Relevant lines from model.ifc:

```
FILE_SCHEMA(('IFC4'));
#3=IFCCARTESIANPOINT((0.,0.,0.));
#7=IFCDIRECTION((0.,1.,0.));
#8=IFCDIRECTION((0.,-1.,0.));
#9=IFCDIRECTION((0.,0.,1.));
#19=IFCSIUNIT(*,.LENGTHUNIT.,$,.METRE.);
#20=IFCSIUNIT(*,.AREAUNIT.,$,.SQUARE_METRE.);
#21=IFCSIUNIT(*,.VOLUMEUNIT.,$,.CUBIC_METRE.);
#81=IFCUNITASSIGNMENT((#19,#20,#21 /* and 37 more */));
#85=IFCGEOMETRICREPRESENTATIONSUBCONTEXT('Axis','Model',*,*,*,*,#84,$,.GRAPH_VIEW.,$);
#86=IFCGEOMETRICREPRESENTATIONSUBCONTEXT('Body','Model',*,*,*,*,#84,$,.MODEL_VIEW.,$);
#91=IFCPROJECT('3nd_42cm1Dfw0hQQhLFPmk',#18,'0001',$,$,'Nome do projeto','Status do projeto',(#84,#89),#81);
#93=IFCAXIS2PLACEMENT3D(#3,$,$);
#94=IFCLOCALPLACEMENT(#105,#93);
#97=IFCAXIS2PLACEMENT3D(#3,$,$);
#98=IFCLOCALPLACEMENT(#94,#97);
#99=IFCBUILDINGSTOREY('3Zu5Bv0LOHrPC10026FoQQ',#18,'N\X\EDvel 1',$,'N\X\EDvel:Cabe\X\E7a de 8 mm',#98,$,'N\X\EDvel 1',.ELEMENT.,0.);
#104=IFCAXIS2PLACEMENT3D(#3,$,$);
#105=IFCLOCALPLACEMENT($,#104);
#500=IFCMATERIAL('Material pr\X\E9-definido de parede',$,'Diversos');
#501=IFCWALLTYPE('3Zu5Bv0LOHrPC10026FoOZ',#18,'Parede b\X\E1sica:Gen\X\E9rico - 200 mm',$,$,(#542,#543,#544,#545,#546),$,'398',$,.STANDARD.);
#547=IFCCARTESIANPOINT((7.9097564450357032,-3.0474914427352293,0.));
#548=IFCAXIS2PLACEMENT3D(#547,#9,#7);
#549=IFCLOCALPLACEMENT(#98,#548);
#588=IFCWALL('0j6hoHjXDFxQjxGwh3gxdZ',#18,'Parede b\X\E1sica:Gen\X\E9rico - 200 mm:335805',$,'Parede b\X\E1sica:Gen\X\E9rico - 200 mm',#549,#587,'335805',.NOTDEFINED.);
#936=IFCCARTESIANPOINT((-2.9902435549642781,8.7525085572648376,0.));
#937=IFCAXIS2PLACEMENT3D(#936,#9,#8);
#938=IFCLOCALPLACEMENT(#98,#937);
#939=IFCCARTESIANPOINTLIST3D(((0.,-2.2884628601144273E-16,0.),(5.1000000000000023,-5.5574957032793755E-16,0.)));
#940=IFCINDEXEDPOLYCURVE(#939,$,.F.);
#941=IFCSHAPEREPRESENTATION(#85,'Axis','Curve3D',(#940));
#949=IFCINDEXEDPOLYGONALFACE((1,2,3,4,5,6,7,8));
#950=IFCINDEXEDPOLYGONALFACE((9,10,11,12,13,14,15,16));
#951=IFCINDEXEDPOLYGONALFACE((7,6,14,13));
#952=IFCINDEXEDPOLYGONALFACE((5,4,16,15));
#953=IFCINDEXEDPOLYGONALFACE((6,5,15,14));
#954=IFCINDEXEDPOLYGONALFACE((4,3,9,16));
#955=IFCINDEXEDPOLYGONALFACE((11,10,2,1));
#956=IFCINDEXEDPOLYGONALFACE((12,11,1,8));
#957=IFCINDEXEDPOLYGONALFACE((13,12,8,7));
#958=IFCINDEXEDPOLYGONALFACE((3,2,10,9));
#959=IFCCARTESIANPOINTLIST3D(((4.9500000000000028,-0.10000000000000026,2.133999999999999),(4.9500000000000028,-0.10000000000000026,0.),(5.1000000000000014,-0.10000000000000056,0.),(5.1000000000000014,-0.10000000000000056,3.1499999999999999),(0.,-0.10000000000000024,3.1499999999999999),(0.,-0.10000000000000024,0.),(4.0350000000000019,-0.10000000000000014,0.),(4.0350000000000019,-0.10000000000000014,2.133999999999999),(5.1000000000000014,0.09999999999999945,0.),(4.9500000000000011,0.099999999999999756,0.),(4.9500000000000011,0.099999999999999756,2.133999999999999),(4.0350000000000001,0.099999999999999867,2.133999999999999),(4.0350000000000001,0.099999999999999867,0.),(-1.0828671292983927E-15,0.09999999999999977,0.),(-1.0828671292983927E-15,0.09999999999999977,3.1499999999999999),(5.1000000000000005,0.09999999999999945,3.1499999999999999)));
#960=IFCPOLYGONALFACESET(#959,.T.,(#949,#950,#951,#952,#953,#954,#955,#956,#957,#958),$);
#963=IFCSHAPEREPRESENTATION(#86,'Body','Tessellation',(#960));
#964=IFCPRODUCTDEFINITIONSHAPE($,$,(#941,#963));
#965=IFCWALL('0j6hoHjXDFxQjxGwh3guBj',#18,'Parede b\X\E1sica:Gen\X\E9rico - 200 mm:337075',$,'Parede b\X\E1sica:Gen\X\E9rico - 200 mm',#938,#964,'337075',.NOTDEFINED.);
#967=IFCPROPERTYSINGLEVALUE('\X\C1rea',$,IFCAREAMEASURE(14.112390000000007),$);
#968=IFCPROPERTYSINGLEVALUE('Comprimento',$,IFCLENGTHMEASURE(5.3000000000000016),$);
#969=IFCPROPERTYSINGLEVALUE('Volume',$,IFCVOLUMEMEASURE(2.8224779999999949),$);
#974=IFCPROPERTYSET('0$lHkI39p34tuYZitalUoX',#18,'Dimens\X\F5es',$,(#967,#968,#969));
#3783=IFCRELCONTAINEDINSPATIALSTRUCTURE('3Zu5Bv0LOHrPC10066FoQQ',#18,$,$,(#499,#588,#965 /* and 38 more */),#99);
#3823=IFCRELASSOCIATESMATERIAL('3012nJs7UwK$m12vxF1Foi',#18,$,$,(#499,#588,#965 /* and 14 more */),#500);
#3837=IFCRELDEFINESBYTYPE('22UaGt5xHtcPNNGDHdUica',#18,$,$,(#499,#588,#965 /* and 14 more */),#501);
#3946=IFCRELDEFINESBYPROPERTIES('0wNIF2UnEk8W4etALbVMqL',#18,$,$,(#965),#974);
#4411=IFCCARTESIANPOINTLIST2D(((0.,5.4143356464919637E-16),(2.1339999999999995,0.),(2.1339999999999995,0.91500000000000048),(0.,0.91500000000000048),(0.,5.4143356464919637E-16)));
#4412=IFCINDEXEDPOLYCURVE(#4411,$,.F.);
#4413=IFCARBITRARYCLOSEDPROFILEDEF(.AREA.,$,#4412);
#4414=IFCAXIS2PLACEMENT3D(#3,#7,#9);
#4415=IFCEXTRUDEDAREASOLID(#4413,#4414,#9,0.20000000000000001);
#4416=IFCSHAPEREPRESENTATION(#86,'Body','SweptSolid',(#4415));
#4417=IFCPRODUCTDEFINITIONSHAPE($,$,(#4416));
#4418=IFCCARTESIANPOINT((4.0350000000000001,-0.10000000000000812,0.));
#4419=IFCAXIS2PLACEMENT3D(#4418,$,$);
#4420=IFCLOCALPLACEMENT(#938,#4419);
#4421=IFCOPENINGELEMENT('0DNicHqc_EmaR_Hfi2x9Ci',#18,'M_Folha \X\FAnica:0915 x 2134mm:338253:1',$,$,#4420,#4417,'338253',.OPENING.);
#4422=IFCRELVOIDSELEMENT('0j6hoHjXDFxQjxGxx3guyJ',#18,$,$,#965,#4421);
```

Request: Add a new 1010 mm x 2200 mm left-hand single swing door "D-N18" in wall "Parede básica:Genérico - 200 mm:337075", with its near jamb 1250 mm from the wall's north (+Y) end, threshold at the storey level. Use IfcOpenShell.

```python
import numpy as np
import ifcopenshell
import ifcopenshell.api.feature
import ifcopenshell.api.geometry
import ifcopenshell.api.pset
import ifcopenshell.api.root
import ifcopenshell.api.spatial
import ifcopenshell.geom
import ifcopenshell.util.element
import ifcopenshell.util.placement
import ifcopenshell.util.representation
import ifcopenshell.util.shape
import ifcopenshell.util.unit

model = ifcopenshell.open("model.ifc")
unit_scale = ifcopenshell.util.unit.calculate_unit_scale(model)
area_scale = ifcopenshell.util.unit.calculate_unit_scale(model, "AREAUNIT")
volume_scale = ifcopenshell.util.unit.calculate_unit_scale(model, "VOLUMEUNIT")
settings = ifcopenshell.geom.settings()


def volume(element):
    """Net volume in cubic metres, openings subtracted."""
    shape = ifcopenshell.geom.create_shape(settings, element)
    return ifcopenshell.util.shape.get_volume(shape.geometry)


wall = model.by_guid("0j6hoHjXDFxQjxGwh3guBj")
storey = ifcopenshell.util.element.get_container(wall, ifc_class="IfcBuildingStorey")
context = ifcopenshell.util.representation.get_context(model, "Model", "Body", "MODEL_VIEW")
before = volume(wall)

width, height, from_end, sill = 1.01, 2.2, 1.25, 0.0  # metres

# The wall runs along its own X axis, and the end named is its -X end.
wall_shape = ifcopenshell.geom.create_shape(settings, wall)
x, y, z = ifcopenshell.util.shape.get_vertices(wall_shape.geometry).T
start = x.min() + from_end
face, thickness = float(y.min()), float(y.max() - y.min())
wall_matrix = ifcopenshell.util.placement.get_local_placement(wall.ObjectPlacement)
level = ifcopenshell.util.placement.get_local_placement(storey.ObjectPlacement)[2, 3]


def in_wall(x, y):
    """Placement at x, y metres in the wall's axes, at sill height."""
    matrix = wall_matrix.copy()
    matrix[:, 3] = wall_matrix @ np.array([x / unit_scale, y / unit_scale, 0.0, 1.0])
    matrix[2, 3] = level + sill / unit_scale
    return matrix


# Opening: a box that overshoots both wall faces by 50 mm.
opening = ifcopenshell.api.root.create_entity(model, ifc_class="IfcOpeningElement", predefined_type="OPENING")
box = ifcopenshell.api.geometry.add_wall_representation(
    model, context=context, length=width, height=height, thickness=thickness + 0.1
)
ifcopenshell.api.geometry.assign_representation(model, product=opening, representation=box)
ifcopenshell.api.geometry.edit_object_placement(model, product=opening, matrix=in_wall(start, face - 0.05), is_si=False)
ifcopenshell.api.feature.add_feature(model, feature=opening, element=wall)

door = ifcopenshell.api.root.create_entity(model, ifc_class="IfcDoor", name="D-N18", predefined_type="DOOR")
door.OverallWidth, door.OverallHeight = width / unit_scale, height / unit_scale
door.OperationType = "SINGLE_SWING_LEFT"
body = ifcopenshell.api.geometry.add_door_representation(
    model,
    context=context,
    overall_width=door.OverallWidth,
    overall_height=door.OverallHeight,
    operation_type="SINGLE_SWING_LEFT",
    lining_properties={"LiningDepth": thickness / unit_scale, "ThresholdDepth": thickness / unit_scale},
)
ifcopenshell.api.geometry.assign_representation(model, product=door, representation=body)
ifcopenshell.api.spatial.assign_container(model, products=[door], relating_structure=storey)
ifcopenshell.api.feature.add_filling(model, opening=opening, element=door)

# The lining spans the wall, so the door starts at the wall face.
ifcopenshell.api.geometry.edit_object_placement(model, product=door, matrix=in_wall(start, face), is_si=False)

after = volume(wall)

# Update the wall's stored quantities.
pset = model.by_id(ifcopenshell.util.element.get_pset(wall, "Dimensões", should_inherit=False)["id"])
ifcopenshell.api.pset.edit_pset(model, pset=pset, properties={
    "Área": model.create_entity("IfcAreaMeasure", after / thickness / area_scale),
    "Volume": model.create_entity("IfcVolumeMeasure", after / volume_scale),
})

print(f"wall volume {before:.3f} -> {after:.3f} m3")

model.write("model_v2.ifc")
```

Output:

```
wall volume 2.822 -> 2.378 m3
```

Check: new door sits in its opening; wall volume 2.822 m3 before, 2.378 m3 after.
